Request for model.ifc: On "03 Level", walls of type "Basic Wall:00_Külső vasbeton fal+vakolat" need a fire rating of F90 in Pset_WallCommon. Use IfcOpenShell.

First a look at what the model holds.

```python
import ifcopenshell
import ifcopenshell.util.element

model = ifcopenshell.open("model.ifc")
print(model.schema)
storey = next(s for s in model.by_type("IfcBuildingStorey") if s.Name == "03 Level")
walls = [e for e in ifcopenshell.util.element.get_decomposition(storey) if e.is_a("IfcWall")]
seen = {}
for e in walls:
    element_type = ifcopenshell.util.element.get_type(e)
    key = (element_type.Name if element_type != e and element_type else None, ifcopenshell.util.element.get_pset(e, "Pset_WallCommon", "FireRating"))
    seen[key] = seen.get(key, 0) + 1
for (name, value), count in sorted(seen.items(), key=str):
    print(count, "x", name, "|", value)
```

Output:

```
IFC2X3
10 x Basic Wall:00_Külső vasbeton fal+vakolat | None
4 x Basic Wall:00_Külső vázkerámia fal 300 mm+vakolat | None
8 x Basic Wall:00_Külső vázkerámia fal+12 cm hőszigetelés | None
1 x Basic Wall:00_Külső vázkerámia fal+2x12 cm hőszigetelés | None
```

```python
import ifcopenshell
import ifcopenshell.api.pset
import ifcopenshell.util.element

model = ifcopenshell.open("model.ifc")

storey = next(s for s in model.by_type("IfcBuildingStorey") if s.Name == "03 Level")
walls = [e for e in ifcopenshell.util.element.get_decomposition(storey) if e.is_a("IfcWall")]

count = 0
for e in walls:
    element_type = ifcopenshell.util.element.get_type(e)
    if element_type in (None, e) or element_type.Name != "Basic Wall:00_Külső vasbeton fal+vakolat":
        continue
    # add_pset returns the element's existing set when there is one.
    pset = ifcopenshell.api.pset.add_pset(model, product=e, name="Pset_WallCommon")
    ifcopenshell.api.pset.edit_pset(model, pset=pset, properties={"FireRating": "F90"})
    count += 1

print(count, "walls updated")

model.write("model_rev.ifc")
```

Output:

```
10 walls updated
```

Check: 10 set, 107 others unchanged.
